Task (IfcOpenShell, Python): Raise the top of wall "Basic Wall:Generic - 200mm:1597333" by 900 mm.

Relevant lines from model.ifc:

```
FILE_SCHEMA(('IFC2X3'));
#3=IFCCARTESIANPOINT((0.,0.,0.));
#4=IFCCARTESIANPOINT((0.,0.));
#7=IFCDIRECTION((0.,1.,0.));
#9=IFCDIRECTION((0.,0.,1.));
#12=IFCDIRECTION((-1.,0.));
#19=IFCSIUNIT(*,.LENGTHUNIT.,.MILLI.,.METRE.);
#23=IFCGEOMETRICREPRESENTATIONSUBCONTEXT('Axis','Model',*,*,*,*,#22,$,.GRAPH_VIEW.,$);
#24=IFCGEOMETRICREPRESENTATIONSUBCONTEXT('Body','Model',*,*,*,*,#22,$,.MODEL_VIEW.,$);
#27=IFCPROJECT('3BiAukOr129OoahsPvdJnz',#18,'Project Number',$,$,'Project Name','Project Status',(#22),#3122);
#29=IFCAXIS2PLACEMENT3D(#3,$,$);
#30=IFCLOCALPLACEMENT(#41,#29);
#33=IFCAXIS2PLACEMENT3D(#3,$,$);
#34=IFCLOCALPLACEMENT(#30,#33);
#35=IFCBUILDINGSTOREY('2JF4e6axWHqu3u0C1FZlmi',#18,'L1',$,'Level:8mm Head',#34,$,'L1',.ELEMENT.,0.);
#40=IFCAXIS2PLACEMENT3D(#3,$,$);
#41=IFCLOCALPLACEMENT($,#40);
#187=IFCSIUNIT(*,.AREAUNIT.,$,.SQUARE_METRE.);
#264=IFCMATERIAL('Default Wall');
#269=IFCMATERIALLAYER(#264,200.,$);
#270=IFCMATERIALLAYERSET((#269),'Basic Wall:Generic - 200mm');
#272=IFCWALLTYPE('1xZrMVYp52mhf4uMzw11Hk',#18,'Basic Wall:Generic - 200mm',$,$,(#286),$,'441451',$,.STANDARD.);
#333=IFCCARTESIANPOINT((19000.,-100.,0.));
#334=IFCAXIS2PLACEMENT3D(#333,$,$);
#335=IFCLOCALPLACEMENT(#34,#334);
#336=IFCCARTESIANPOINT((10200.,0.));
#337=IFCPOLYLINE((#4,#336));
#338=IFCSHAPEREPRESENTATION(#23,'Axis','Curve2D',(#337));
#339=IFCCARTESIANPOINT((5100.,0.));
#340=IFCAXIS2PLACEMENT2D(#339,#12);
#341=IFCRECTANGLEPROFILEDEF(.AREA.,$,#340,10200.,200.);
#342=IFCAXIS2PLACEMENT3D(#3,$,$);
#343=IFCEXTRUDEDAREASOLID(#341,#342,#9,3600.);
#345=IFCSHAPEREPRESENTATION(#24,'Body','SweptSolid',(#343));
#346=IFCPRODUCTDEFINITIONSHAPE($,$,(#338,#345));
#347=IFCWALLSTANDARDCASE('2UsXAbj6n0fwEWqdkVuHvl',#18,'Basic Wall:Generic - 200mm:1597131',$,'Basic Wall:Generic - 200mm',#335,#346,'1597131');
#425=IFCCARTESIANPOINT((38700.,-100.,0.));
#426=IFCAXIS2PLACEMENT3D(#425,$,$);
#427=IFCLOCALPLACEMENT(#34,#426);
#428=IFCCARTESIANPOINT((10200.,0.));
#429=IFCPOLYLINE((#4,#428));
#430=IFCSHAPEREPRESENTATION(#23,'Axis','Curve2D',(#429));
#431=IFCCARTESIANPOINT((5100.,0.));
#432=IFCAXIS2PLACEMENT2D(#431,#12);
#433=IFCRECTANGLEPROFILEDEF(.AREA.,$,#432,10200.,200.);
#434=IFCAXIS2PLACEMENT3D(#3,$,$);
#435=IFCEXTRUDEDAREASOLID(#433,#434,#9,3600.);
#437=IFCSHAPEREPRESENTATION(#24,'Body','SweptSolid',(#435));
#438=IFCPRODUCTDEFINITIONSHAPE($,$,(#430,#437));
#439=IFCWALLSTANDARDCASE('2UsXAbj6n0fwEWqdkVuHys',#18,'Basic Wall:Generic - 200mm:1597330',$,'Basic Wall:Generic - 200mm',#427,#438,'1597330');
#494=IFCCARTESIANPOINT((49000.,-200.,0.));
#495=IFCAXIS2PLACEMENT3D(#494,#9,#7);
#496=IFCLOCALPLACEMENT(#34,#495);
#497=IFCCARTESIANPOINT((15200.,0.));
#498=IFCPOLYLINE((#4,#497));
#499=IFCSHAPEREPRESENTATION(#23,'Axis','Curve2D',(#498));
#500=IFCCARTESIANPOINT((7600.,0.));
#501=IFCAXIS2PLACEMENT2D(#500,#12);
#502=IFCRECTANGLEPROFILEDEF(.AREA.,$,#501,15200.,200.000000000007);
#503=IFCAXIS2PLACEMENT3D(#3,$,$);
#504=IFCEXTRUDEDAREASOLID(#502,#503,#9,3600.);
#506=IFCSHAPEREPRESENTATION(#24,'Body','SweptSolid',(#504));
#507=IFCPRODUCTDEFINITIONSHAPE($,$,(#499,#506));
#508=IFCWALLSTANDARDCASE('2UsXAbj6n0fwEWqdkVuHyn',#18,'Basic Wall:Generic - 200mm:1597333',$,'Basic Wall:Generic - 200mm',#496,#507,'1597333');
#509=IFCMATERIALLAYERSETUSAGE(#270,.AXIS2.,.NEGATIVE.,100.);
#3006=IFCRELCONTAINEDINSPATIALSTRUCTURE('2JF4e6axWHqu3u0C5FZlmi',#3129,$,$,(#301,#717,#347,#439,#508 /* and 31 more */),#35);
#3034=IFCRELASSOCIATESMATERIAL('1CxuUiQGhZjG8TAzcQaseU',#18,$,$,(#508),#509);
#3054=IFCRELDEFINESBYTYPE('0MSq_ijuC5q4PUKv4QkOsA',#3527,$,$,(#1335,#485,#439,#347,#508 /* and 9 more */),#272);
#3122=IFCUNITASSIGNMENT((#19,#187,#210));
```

```python
import ifcopenshell
import ifcopenshell.geom
import ifcopenshell.util.representation
import ifcopenshell.util.shape
import ifcopenshell.util.unit

model = ifcopenshell.open("model.ifc")
unit_scale = ifcopenshell.util.unit.calculate_unit_scale(model)
settings = ifcopenshell.geom.settings()


def volume(element):
    """Net volume in cubic metres, openings subtracted."""
    shape = ifcopenshell.geom.create_shape(settings, element)
    return ifcopenshell.util.shape.get_volume(shape.geometry)


wall = model.by_guid("2UsXAbj6n0fwEWqdkVuHyn")
before = volume(wall)

body = ifcopenshell.util.representation.get_representation(wall, "Model", "Body")
solid = body.Items[0]
old_height = solid.Depth
solid.Depth += 0.9 / unit_scale
after = volume(wall)

print(f"height {old_height:g} -> {solid.Depth:g}, volume {before:.3f} -> {after:.3f} m3")

model.write("model-out.ifc")
```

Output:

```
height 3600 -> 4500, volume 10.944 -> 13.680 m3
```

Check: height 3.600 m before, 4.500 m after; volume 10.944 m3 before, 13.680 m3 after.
